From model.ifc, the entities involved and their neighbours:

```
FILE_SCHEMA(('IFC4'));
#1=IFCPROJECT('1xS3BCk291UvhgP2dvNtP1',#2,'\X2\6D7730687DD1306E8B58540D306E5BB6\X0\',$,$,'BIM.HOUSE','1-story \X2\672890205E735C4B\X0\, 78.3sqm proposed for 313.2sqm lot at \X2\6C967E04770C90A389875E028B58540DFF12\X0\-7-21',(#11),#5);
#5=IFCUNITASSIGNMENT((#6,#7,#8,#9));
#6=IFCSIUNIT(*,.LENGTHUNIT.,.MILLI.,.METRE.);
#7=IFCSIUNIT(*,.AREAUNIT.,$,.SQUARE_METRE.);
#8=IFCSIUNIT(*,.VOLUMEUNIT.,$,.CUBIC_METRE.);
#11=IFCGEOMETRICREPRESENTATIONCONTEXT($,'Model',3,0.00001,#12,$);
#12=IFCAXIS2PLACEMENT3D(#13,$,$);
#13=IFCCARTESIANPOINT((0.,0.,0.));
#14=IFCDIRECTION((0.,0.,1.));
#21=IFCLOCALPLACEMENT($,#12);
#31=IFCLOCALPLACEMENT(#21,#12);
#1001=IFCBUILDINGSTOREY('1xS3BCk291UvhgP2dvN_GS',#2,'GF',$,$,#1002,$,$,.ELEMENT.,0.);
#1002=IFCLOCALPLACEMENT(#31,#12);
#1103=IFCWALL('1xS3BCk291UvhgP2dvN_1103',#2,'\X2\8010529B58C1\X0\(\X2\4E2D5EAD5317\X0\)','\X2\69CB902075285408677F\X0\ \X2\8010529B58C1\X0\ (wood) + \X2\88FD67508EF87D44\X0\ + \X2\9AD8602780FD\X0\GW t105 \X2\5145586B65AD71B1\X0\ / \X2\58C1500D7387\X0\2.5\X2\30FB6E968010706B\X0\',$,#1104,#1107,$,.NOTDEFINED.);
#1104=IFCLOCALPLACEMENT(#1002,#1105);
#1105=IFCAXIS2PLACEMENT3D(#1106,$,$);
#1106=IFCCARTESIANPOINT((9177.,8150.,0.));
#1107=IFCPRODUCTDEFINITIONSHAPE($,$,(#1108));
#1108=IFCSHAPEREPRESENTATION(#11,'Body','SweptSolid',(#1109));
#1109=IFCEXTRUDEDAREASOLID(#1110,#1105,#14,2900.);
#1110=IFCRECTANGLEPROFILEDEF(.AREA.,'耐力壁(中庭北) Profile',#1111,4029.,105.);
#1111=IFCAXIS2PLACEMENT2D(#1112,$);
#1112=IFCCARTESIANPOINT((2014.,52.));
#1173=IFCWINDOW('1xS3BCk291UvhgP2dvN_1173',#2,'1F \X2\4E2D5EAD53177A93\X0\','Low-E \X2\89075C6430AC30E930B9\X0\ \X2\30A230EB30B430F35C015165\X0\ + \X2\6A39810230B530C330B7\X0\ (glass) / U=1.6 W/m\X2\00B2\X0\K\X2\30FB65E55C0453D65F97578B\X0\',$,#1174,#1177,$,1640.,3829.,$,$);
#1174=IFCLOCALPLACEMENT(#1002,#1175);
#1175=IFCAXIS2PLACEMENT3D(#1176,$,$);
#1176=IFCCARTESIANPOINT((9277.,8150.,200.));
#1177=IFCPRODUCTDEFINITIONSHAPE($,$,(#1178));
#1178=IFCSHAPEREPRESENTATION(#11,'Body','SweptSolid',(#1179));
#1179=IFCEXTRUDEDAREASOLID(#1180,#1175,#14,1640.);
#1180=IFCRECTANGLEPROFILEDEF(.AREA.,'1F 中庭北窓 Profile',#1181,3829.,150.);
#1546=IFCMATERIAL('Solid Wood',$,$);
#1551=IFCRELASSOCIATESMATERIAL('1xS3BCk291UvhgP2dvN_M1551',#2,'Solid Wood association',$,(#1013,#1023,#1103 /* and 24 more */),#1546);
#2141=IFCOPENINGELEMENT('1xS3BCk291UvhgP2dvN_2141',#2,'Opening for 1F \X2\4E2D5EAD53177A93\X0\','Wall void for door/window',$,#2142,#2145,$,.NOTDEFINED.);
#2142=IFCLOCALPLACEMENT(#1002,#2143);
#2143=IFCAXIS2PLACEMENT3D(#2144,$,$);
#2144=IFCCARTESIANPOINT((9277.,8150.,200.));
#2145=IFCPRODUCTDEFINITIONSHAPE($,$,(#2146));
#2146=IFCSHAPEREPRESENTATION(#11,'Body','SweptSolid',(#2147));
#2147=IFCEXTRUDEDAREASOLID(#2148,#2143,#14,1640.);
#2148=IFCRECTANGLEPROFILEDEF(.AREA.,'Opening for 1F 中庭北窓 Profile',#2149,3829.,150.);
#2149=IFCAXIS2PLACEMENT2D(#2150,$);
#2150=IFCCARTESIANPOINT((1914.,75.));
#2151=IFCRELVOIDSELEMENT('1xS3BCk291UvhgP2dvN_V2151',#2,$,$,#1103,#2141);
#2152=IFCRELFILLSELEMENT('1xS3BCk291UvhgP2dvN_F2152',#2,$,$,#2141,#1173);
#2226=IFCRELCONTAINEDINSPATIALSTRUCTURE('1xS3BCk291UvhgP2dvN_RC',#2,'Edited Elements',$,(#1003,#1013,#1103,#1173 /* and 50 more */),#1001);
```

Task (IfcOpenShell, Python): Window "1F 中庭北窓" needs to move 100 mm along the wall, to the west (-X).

```python
import ifcopenshell
import ifcopenshell.api.geometry
import ifcopenshell.util.placement
import ifcopenshell.util.unit

model = ifcopenshell.open("model.ifc")
unit_scale = ifcopenshell.util.unit.calculate_unit_scale(model)

window = model.by_guid("1xS3BCk291UvhgP2dvN_1173")
opening = window.FillsVoids[0].RelatingOpeningElement
wall = opening.VoidsElements[0].RelatingBuildingElement

wall_matrix = ifcopenshell.util.placement.get_local_placement(wall.ObjectPlacement)
shift = wall_matrix[:3, 0] * -0.1 / unit_scale
before = ifcopenshell.util.placement.get_local_placement(window.ObjectPlacement)[:3, 3].copy()

# The window is not placed relative to its opening, so move both.
for product in (opening, window):
    matrix = ifcopenshell.util.placement.get_local_placement(product.ObjectPlacement)
    matrix[:3, 3] += shift
    ifcopenshell.api.geometry.edit_object_placement(model, product=product, matrix=matrix, is_si=False)

after = ifcopenshell.util.placement.get_local_placement(window.ObjectPlacement)[:3, 3]
print("window moved by", (after - before).round(3) + 0.0)

model.write("model_updated.ifc")
```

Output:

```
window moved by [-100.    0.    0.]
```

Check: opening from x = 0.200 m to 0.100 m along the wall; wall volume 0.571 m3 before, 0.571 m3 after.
